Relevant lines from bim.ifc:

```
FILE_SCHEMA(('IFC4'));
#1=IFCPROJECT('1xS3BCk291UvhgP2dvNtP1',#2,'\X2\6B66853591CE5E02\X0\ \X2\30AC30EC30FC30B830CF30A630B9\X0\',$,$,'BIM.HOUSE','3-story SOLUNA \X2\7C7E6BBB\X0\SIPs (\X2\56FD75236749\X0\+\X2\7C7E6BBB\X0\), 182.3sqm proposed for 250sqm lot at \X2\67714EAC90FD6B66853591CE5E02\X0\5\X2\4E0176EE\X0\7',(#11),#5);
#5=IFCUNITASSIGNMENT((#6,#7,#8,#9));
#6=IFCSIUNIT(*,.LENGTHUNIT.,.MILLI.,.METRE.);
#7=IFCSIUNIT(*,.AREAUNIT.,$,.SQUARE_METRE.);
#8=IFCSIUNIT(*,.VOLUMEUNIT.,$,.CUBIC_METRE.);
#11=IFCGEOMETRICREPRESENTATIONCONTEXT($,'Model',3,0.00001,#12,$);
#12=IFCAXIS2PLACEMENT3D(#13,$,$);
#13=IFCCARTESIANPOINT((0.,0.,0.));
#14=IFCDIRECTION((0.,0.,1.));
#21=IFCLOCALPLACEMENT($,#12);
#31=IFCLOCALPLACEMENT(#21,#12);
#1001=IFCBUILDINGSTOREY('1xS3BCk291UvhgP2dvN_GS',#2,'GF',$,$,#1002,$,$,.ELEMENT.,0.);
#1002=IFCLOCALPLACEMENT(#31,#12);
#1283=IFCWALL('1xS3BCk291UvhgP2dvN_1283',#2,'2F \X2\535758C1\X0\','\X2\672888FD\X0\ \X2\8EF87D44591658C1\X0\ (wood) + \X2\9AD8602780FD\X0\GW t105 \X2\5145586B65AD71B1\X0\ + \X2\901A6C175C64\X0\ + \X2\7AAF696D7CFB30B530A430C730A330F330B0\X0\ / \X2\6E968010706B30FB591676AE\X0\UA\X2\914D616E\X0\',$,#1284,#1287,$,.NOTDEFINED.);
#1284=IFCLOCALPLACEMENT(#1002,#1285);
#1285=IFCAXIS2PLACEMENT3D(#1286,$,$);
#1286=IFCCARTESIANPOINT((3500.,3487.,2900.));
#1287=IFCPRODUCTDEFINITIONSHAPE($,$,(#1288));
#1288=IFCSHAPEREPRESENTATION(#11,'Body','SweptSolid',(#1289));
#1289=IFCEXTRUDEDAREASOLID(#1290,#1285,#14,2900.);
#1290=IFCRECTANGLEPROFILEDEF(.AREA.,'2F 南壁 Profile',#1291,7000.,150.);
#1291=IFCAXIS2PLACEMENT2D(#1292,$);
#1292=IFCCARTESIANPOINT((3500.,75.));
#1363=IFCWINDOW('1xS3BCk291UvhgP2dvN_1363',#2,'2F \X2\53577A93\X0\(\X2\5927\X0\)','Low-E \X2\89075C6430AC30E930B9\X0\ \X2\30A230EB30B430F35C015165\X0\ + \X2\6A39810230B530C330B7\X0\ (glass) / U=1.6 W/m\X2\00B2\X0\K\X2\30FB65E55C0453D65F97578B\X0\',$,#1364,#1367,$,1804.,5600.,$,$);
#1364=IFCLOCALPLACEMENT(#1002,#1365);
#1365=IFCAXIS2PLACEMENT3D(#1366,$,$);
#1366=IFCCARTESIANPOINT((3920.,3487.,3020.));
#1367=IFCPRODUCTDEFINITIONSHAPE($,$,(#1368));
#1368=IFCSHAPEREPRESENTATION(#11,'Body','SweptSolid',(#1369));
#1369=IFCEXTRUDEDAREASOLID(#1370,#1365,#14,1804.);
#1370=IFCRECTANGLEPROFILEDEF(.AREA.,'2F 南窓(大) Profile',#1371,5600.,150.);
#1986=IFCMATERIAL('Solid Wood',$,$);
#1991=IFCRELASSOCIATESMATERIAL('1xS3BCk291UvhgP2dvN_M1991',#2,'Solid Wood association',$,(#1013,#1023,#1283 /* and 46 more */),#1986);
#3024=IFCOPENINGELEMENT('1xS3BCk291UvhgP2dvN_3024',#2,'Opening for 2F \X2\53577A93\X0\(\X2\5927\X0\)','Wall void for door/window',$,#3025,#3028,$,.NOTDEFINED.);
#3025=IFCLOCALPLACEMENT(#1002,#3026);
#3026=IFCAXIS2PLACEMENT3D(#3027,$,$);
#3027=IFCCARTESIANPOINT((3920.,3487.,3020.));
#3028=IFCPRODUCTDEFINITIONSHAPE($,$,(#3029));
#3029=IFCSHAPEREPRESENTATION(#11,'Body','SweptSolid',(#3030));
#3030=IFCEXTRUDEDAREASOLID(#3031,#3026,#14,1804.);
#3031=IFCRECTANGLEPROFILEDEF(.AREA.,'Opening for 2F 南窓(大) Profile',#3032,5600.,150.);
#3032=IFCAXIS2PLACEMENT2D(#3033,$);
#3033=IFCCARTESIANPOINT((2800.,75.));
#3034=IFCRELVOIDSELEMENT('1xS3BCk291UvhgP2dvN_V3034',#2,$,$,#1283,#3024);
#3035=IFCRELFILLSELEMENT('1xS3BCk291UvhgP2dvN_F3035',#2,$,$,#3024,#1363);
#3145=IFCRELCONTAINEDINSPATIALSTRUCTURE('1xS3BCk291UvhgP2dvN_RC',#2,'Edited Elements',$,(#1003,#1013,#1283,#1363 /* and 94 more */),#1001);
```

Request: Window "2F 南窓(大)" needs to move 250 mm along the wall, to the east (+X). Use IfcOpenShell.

```python
import ifcopenshell
import ifcopenshell.api.geometry
import ifcopenshell.util.placement

model = ifcopenshell.open("bim.ifc")

window = model.by_id(1363)
opening = window.FillsVoids[0].RelatingOpeningElement
wall = opening.VoidsElements[0].RelatingBuildingElement

wall_matrix = ifcopenshell.util.placement.get_local_placement(wall.ObjectPlacement)
shift = wall_matrix[:3, 0] * 250.0
before = ifcopenshell.util.placement.get_local_placement(window.ObjectPlacement)[:3, 3].copy()

# The window is not placed relative to its opening, so move both.
for product in (opening, window):
    matrix = ifcopenshell.util.placement.get_local_placement(product.ObjectPlacement)
    matrix[:3, 3] += shift
    ifcopenshell.api.geometry.edit_object_placement(model, product=product, matrix=matrix, is_si=False)

after = ifcopenshell.util.placement.get_local_placement(window.ObjectPlacement)[:3, 3]
print("window moved by", (after - before).round(3) + 0.0)

model.write("bim_v2.ifc")
```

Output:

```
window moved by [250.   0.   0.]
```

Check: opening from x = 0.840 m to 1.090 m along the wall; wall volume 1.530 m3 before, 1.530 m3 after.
